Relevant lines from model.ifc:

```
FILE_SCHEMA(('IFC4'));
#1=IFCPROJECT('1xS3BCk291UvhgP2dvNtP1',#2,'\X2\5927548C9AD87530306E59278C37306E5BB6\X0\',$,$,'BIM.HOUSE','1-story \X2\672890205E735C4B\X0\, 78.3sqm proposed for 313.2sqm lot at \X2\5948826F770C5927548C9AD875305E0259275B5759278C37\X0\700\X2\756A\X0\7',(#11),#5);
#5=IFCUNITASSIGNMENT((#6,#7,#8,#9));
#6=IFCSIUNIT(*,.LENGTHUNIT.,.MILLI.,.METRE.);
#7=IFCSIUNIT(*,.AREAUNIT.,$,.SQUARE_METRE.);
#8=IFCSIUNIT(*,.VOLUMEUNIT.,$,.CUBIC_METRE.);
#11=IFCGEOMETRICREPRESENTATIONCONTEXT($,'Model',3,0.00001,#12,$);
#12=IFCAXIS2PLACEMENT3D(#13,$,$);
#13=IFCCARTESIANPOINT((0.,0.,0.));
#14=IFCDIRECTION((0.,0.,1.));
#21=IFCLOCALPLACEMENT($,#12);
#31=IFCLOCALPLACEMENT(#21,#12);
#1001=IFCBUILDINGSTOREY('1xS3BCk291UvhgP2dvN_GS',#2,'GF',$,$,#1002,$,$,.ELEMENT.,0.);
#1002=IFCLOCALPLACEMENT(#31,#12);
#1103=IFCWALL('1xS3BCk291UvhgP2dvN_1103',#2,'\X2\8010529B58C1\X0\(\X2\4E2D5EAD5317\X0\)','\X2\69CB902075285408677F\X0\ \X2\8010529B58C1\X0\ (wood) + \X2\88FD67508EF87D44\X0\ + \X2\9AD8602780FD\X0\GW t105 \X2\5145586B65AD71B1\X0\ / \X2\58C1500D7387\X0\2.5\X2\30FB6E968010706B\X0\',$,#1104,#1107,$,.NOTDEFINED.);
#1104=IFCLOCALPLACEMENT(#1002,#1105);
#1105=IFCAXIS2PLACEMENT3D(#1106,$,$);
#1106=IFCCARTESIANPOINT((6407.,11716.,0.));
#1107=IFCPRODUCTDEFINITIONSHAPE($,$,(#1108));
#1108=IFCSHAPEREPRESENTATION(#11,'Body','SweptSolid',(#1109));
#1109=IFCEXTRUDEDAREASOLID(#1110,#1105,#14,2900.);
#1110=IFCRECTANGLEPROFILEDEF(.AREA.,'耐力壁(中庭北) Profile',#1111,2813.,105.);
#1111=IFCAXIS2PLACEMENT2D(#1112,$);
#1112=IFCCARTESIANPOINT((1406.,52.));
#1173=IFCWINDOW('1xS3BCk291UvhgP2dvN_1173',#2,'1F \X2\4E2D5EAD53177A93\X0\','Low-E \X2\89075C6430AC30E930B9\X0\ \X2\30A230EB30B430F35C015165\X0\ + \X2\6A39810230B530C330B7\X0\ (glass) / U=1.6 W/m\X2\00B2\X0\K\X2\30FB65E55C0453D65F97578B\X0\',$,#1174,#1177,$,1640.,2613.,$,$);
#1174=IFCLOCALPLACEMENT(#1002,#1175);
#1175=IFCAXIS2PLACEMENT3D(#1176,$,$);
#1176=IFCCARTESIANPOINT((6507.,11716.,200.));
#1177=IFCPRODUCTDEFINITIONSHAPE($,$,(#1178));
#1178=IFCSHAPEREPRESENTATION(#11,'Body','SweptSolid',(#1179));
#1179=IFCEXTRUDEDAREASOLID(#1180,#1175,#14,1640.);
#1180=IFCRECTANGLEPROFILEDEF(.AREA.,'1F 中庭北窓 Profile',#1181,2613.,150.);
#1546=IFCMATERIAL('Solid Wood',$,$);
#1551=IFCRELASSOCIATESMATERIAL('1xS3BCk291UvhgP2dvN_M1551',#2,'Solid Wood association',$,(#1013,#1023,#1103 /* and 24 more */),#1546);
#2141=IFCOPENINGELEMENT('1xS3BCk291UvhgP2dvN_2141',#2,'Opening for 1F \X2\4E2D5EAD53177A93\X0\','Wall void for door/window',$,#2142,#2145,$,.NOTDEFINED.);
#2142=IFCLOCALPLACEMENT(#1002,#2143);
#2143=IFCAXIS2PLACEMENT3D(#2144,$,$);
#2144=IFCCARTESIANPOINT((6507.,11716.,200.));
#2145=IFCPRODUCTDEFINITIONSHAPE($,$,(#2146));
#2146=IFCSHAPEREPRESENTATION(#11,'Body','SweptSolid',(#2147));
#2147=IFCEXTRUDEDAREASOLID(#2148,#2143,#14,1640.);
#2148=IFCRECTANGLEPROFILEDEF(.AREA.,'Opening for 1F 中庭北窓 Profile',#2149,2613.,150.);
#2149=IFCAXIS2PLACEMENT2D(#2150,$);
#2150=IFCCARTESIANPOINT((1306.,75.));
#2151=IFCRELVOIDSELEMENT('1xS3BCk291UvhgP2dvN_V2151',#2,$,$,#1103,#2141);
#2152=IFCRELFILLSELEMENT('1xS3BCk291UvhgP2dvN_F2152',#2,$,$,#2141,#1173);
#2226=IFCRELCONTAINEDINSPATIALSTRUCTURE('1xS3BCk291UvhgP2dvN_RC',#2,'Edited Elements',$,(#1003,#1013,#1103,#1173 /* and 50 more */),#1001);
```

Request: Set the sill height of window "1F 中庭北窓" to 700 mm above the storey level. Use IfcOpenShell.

```python
import numpy as np
import ifcopenshell
import ifcopenshell.api.geometry
import ifcopenshell.geom
import ifcopenshell.util.element
import ifcopenshell.util.placement
import ifcopenshell.util.shape
import ifcopenshell.util.unit

model = ifcopenshell.open("model.ifc")
unit_scale = ifcopenshell.util.unit.calculate_unit_scale(model)

window = model.by_guid("1xS3BCk291UvhgP2dvN_1173")
opening = window.FillsVoids[0].RelatingOpeningElement
storey = ifcopenshell.util.element.get_container(window, ifc_class="IfcBuildingStorey")
level = ifcopenshell.util.placement.get_local_placement(storey.ObjectPlacement)[2, 3]

# The opening's origin need not be at the sill, so measure its lowest point.
shape = ifcopenshell.geom.create_shape(ifcopenshell.geom.settings(), opening)
bottom = ifcopenshell.util.shape.get_shape_bottom_elevation(shape, shape.geometry) / unit_scale
dz = level + 700.0 - bottom

shift = np.array([0.0, 0.0, dz])
# The window is not placed relative to its opening, so move both.
for product in (opening, window):
    matrix = ifcopenshell.util.placement.get_local_placement(product.ObjectPlacement)
    matrix[:3, 3] += shift
    ifcopenshell.api.geometry.edit_object_placement(model, product=product, matrix=matrix, is_si=False)

print(f"moved by {dz * unit_scale:+.3f} m")

model.write("model_v2.ifc")
```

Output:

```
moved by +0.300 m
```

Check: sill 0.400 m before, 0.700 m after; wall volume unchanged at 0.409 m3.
